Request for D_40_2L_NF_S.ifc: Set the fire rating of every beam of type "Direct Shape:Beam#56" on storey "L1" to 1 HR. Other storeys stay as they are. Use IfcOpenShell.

First a look at what the model holds.

```python
import ifcopenshell
import ifcopenshell.util.element

model = ifcopenshell.open("D_40_2L_NF_S.ifc")
print(model.schema)
storey = next(s for s in model.by_type("IfcBuildingStorey") if s.Name == "L1")
beams = [e for e in ifcopenshell.util.element.get_decomposition(storey) if e.is_a("IfcBeam")]
seen = {}
for e in beams:
    element_type = ifcopenshell.util.element.get_type(e)
    key = (element_type.Name if element_type != e and element_type else None, ifcopenshell.util.element.get_pset(e, "Pset_BeamCommon", "FireRating"))
    seen[key] = seen.get(key, 0) + 1
for (name, value), count in sorted(seen.items(), key=str):
    print(count, "x", name, "|", value)
```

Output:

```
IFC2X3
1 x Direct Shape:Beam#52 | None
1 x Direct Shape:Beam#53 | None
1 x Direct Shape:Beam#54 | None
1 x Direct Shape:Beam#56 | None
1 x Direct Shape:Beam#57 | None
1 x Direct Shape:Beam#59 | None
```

```python
import ifcopenshell
import ifcopenshell.api.pset
import ifcopenshell.util.element

model = ifcopenshell.open("D_40_2L_NF_S.ifc")

storey = next(s for s in model.by_type("IfcBuildingStorey") if s.Name == "L1")
beams = [e for e in ifcopenshell.util.element.get_decomposition(storey) if e.is_a("IfcBeam")]

count = 0
for e in beams:
    element_type = ifcopenshell.util.element.get_type(e)
    if element_type in (None, e) or element_type.Name != "Direct Shape:Beam#56":
        continue
    # add_pset returns the element's existing set when there is one.
    pset = ifcopenshell.api.pset.add_pset(model, product=e, name="Pset_BeamCommon")
    ifcopenshell.api.pset.edit_pset(model, pset=pset, properties={"FireRating": "1 HR"})
    count += 1

print(count, "beams updated")

model.write("D_40_2L_NF_S_edited.ifc")
```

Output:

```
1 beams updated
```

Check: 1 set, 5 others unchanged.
